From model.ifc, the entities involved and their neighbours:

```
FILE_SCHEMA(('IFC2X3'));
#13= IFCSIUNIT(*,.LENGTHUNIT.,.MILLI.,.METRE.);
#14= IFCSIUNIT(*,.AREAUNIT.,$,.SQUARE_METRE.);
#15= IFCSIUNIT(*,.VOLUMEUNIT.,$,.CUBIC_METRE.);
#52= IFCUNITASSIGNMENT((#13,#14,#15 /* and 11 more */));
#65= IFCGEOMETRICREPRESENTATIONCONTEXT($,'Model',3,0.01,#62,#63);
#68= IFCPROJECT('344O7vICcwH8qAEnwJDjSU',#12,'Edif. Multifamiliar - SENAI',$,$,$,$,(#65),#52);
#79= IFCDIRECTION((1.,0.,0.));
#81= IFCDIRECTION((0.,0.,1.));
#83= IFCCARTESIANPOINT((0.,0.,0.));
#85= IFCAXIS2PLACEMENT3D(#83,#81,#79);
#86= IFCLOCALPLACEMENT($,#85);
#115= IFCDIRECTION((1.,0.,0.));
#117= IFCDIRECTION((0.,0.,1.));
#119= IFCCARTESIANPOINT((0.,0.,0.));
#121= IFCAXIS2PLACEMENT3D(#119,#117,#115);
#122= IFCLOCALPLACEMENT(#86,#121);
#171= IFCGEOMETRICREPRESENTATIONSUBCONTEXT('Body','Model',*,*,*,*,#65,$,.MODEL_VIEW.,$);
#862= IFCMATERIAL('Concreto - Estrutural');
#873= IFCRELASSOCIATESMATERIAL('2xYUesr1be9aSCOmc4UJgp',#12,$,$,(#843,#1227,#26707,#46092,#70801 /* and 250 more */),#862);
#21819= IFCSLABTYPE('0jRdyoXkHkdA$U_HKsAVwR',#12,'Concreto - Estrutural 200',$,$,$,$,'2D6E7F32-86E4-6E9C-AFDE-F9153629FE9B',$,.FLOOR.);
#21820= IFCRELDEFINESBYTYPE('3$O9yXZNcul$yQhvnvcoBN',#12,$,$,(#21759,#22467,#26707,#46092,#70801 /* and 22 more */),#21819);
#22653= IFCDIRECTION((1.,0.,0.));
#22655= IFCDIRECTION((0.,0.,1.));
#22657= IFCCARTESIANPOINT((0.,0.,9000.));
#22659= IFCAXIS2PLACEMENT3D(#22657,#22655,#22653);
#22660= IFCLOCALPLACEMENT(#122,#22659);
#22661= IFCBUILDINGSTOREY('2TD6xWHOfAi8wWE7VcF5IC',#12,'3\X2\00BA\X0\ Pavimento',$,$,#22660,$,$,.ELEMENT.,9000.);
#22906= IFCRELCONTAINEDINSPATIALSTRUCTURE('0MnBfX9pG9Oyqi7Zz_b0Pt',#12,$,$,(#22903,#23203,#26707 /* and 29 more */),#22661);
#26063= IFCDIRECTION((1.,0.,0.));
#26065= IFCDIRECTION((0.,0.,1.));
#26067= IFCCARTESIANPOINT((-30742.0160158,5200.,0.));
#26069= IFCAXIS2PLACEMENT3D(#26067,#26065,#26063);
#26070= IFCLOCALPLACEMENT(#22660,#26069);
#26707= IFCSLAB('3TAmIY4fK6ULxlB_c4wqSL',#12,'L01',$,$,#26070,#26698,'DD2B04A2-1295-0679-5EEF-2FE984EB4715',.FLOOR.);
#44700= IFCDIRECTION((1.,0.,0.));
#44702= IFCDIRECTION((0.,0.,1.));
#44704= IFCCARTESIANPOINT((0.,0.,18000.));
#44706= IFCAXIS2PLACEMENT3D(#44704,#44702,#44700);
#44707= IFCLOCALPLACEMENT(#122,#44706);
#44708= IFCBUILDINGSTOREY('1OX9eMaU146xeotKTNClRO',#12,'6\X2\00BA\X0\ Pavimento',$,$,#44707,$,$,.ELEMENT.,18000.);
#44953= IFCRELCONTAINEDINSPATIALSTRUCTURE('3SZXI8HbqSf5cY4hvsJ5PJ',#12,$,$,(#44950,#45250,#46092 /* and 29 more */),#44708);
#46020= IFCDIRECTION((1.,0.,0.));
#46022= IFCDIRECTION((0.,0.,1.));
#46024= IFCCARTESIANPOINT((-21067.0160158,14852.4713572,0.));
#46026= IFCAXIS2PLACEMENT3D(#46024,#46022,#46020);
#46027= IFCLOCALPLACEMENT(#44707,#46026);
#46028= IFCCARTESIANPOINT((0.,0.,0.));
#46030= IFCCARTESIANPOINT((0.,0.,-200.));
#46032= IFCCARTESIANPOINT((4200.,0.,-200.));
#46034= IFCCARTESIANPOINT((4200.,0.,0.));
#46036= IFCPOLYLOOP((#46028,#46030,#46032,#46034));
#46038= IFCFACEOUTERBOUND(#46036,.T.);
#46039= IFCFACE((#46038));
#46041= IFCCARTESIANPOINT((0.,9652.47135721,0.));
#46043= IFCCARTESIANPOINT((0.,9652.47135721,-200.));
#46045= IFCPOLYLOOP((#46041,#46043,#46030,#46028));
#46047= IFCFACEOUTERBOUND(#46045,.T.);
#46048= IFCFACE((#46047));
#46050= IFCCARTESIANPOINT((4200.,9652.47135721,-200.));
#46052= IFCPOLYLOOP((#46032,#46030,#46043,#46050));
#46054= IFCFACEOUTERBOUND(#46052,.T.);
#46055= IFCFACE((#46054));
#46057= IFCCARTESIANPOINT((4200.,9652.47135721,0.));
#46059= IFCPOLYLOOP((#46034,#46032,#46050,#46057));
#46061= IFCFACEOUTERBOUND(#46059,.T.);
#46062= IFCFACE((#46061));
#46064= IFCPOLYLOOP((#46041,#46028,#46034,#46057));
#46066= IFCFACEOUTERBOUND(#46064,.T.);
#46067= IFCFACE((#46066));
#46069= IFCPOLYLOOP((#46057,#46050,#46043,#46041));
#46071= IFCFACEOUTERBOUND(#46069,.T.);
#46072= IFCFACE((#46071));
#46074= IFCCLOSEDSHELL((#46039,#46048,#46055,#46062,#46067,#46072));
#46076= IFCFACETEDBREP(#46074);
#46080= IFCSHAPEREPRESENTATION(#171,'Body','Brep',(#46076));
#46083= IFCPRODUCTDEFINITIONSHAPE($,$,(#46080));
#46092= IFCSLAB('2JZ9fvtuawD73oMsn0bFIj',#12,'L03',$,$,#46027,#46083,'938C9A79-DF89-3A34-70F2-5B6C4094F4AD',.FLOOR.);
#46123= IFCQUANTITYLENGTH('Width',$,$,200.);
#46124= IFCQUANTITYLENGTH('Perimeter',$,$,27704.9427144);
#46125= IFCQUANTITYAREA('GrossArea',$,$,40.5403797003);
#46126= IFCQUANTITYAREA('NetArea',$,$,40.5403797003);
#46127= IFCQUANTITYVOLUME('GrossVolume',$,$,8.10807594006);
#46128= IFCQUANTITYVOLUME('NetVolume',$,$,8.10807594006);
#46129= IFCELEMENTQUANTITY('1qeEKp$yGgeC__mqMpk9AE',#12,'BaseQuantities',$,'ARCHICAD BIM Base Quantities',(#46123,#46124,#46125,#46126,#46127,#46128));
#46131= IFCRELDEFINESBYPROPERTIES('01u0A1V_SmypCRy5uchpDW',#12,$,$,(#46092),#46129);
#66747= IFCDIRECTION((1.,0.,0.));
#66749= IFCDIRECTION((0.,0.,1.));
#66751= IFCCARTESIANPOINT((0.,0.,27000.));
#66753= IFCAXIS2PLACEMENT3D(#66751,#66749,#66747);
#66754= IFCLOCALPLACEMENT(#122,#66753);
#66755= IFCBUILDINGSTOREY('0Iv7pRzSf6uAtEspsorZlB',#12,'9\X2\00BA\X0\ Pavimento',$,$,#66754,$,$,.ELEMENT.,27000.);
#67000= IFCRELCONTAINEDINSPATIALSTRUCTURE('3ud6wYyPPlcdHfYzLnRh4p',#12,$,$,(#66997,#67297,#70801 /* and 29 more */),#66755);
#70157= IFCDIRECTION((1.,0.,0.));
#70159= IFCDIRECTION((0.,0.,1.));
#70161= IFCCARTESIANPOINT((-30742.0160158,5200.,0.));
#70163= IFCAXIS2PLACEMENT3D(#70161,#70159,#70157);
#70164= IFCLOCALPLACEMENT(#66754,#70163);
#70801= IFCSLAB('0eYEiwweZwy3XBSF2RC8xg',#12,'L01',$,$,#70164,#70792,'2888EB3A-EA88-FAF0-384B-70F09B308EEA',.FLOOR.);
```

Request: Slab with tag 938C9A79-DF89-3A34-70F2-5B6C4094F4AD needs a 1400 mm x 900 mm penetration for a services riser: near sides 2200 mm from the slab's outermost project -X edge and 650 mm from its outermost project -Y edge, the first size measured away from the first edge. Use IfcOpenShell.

```python
import numpy as np
import ifcopenshell
import ifcopenshell.api.feature
import ifcopenshell.api.geometry
import ifcopenshell.api.pset
import ifcopenshell.api.root
import ifcopenshell.geom
import ifcopenshell.util.element
import ifcopenshell.util.placement
import ifcopenshell.util.representation
import ifcopenshell.util.shape
import ifcopenshell.util.unit

model = ifcopenshell.open("model.ifc")
unit_scale = ifcopenshell.util.unit.calculate_unit_scale(model)
area_scale = ifcopenshell.util.unit.calculate_unit_scale(model, "AREAUNIT")
volume_scale = ifcopenshell.util.unit.calculate_unit_scale(model, "VOLUMEUNIT")
settings = ifcopenshell.geom.settings()


def volume(element):
    """Net volume in cubic metres, openings subtracted."""
    shape = ifcopenshell.geom.create_shape(settings, element)
    return ifcopenshell.util.shape.get_volume(shape.geometry)


slab = model.by_guid("2JZ9fvtuawD73oMsn0bFIj")
before = volume(slab)

# Extent in the slab's own axes, in metres. The edges named are its -X and -Y sides.
slab_shape = ifcopenshell.geom.create_shape(settings, slab)
vertices = ifcopenshell.util.shape.get_vertices(slab_shape.geometry)
x_min, y_min, bottom = vertices.min(axis=0)
top = vertices[:, 2].max()

opening = ifcopenshell.api.root.create_entity(model, ifc_class="IfcOpeningElement", name="Services riser opening")
context = ifcopenshell.util.representation.get_context(model, "Model", "Body", "MODEL_VIEW")
width, depth = 1.4, 0.9
outline = [(0.0, 0.0), (width, 0.0), (width, depth), (0.0, depth), (0.0, 0.0)]
# Overshoot both faces by 50 mm so the cut is clean.
shape = ifcopenshell.api.geometry.add_slab_representation(
    model, context=context, depth=top - bottom + 0.1, polyline=outline
)
ifcopenshell.api.geometry.assign_representation(model, product=opening, representation=shape)

matrix = ifcopenshell.util.placement.get_local_placement(slab.ObjectPlacement)
matrix[:, 3] = matrix @ np.append(np.array([x_min + 2.2, y_min + 0.65, bottom - 0.05]) / unit_scale, 1.0)
ifcopenshell.api.geometry.edit_object_placement(model, product=opening, matrix=matrix, is_si=False)
ifcopenshell.api.feature.add_feature(model, feature=opening, element=slab)

after = volume(slab)

# Update the slab's stored quantities.
qto = model.by_id(ifcopenshell.util.element.get_pset(slab, "BaseQuantities", should_inherit=False)["id"])
ifcopenshell.api.pset.edit_qto(model, qto=qto, properties={
    "NetArea": after / (top - bottom) / area_scale,
    "NetVolume": after / volume_scale,
})

print(f"slab volume {before:.3f} -> {after:.3f} m3")

model.write("model_edited.ifc")
```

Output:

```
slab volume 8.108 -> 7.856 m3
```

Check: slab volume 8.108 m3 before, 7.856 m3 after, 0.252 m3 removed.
